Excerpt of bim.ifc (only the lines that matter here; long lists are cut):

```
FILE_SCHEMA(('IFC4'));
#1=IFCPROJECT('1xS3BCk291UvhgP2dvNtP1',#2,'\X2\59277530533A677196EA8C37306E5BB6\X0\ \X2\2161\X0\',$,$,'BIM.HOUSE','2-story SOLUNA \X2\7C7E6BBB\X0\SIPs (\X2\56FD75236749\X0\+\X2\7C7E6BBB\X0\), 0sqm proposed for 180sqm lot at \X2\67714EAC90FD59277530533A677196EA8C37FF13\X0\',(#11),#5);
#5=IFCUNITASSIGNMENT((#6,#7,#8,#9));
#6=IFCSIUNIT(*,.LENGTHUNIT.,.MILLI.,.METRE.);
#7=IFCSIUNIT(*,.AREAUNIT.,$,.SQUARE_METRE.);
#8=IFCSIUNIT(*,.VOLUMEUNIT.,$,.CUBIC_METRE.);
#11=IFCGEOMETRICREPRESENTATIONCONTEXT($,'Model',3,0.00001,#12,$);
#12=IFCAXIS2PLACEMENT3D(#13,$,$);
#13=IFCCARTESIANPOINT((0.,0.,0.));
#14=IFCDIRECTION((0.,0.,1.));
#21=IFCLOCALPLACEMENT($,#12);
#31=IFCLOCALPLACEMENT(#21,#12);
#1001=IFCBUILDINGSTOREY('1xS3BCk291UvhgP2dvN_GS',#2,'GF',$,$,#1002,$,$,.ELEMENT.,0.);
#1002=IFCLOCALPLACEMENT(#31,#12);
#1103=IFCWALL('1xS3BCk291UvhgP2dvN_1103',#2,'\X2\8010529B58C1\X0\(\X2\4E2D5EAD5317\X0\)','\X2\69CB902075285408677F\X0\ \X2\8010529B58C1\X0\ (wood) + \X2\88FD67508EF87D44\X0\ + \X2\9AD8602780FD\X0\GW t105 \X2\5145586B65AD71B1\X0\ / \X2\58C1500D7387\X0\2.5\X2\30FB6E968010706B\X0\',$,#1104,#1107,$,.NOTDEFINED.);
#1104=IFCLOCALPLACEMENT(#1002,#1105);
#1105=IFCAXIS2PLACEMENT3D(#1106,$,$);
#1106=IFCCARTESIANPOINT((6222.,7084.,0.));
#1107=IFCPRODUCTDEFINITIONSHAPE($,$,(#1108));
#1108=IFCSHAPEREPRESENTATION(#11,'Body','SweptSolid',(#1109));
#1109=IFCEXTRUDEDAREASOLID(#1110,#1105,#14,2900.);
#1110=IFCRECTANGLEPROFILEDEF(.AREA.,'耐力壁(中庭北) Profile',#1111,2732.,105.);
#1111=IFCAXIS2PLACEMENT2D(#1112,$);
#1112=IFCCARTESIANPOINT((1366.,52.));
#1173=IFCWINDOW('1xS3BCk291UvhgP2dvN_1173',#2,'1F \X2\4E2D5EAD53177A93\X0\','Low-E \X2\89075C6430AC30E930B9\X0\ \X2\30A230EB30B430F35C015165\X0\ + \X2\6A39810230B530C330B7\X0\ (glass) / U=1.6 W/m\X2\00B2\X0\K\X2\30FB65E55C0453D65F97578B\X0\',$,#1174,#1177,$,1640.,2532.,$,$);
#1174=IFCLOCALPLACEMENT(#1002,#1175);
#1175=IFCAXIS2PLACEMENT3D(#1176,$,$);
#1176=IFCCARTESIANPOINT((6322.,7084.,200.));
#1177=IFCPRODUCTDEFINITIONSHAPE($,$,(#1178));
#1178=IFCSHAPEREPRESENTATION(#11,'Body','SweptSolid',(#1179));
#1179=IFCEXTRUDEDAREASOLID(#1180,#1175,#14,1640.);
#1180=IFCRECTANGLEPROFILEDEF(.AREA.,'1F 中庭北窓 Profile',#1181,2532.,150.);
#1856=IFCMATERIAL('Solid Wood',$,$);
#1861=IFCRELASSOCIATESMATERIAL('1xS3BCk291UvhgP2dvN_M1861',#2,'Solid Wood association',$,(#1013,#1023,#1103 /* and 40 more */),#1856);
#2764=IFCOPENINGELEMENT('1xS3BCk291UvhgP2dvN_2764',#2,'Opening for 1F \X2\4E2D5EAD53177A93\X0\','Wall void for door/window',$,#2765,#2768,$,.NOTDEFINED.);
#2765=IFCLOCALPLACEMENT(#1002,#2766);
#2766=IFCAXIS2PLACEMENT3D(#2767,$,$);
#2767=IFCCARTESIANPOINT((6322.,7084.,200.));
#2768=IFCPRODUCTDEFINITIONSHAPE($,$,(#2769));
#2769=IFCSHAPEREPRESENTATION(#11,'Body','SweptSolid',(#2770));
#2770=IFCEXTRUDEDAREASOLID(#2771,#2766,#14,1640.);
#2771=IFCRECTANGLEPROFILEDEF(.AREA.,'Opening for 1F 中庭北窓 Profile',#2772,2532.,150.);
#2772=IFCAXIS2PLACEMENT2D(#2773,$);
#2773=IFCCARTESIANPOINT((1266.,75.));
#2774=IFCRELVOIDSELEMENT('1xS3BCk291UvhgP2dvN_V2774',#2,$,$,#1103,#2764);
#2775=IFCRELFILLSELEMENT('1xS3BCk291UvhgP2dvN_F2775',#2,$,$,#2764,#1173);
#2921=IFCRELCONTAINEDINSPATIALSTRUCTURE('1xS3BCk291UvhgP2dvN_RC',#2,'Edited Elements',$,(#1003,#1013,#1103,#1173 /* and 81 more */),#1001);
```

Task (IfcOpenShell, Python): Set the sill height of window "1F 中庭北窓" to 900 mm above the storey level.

```python
import numpy as np
import ifcopenshell
import ifcopenshell.api.geometry
import ifcopenshell.geom
import ifcopenshell.util.element
import ifcopenshell.util.placement
import ifcopenshell.util.shape
import ifcopenshell.util.unit

model = ifcopenshell.open("bim.ifc")
unit_scale = ifcopenshell.util.unit.calculate_unit_scale(model)

window = model.by_guid("1xS3BCk291UvhgP2dvN_1173")
opening = window.FillsVoids[0].RelatingOpeningElement
storey = ifcopenshell.util.element.get_container(window, ifc_class="IfcBuildingStorey")
level = ifcopenshell.util.placement.get_local_placement(storey.ObjectPlacement)[2, 3]

# The opening's origin need not be at the sill, so measure its lowest point.
shape = ifcopenshell.geom.create_shape(ifcopenshell.geom.settings(), opening)
bottom = ifcopenshell.util.shape.get_shape_bottom_elevation(shape, shape.geometry) / unit_scale
dz = level + 900.0 - bottom

shift = np.array([0.0, 0.0, dz])
# The window is not placed relative to its opening, so move both.
for product in (opening, window):
    matrix = ifcopenshell.util.placement.get_local_placement(product.ObjectPlacement)
    matrix[:3, 3] += shift
    ifcopenshell.api.geometry.edit_object_placement(model, product=product, matrix=matrix, is_si=False)

print(f"moved by {dz * unit_scale:+.3f} m")

model.write("bim_updated.ifc")
```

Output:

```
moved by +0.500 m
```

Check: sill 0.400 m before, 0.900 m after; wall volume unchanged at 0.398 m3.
